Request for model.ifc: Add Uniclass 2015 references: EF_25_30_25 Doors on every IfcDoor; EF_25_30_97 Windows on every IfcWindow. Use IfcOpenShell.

First a look at what the model holds.

```python
import ifcopenshell

model = ifcopenshell.open("model.ifc")
print(model.schema)
print("classifications:", [c.Name for c in model.by_type("IfcClassification")])
for ifc_class in ("IfcDoor", "IfcRoof", "IfcStair", "IfcWall", "IfcWindow"):
    print(ifc_class, len(model.by_type(ifc_class)))
```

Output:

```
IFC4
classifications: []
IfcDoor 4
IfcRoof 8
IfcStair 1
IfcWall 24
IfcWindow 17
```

```python
import ifcopenshell
import ifcopenshell.api.classification

model = ifcopenshell.open("model.ifc")

system = ifcopenshell.api.classification.add_classification(model, classification="Uniclass 2015")

codes = {
    "IfcDoor": ("EF_25_30_25", "Doors"),
    "IfcWindow": ("EF_25_30_97", "Windows"),
}
for ifc_class, (code, name) in codes.items():
    products = model.by_type(ifc_class)
    ifcopenshell.api.classification.add_reference(
        model, products=products, classification=system, identification=code, name=name
    )
    print(code, len(products))

model.write("model_edited.ifc")
```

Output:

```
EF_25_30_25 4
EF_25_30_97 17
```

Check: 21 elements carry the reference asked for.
